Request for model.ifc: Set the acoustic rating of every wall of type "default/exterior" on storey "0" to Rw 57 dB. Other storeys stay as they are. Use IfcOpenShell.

First a look at what the model holds.

```python
import ifcopenshell
import ifcopenshell.util.element

model = ifcopenshell.open("model.ifc")
print(model.schema)
storey = next(s for s in model.by_type("IfcBuildingStorey") if s.Name == "0")
walls = [e for e in ifcopenshell.util.element.get_decomposition(storey) if e.is_a("IfcWall")]
seen = {}
for e in walls:
    element_type = ifcopenshell.util.element.get_type(e)
    key = (element_type.Name if element_type != e and element_type else None, ifcopenshell.util.element.get_pset(e, "Pset_WallCommon", "AcousticRating"))
    seen[key] = seen.get(key, 0) + 1
for (name, value), count in sorted(seen.items(), key=str):
    print(count, "x", name, "|", value)
```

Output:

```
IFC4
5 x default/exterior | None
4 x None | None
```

```python
import ifcopenshell
import ifcopenshell.api.pset
import ifcopenshell.util.element

model = ifcopenshell.open("model.ifc")

storey = next(s for s in model.by_type("IfcBuildingStorey") if s.Name == "0")
walls = [e for e in ifcopenshell.util.element.get_decomposition(storey) if e.is_a("IfcWall")]

count = 0
for e in walls:
    element_type = ifcopenshell.util.element.get_type(e)
    if element_type in (None, e) or element_type.Name != "default/exterior":
        continue
    # add_pset returns the element's existing set when there is one.
    pset = ifcopenshell.api.pset.add_pset(model, product=e, name="Pset_WallCommon")
    ifcopenshell.api.pset.edit_pset(model, pset=pset, properties={"AcousticRating": "Rw 57 dB"})
    count += 1

print(count, "walls updated")

model.write("model_edited.ifc")
```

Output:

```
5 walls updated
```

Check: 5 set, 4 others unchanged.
